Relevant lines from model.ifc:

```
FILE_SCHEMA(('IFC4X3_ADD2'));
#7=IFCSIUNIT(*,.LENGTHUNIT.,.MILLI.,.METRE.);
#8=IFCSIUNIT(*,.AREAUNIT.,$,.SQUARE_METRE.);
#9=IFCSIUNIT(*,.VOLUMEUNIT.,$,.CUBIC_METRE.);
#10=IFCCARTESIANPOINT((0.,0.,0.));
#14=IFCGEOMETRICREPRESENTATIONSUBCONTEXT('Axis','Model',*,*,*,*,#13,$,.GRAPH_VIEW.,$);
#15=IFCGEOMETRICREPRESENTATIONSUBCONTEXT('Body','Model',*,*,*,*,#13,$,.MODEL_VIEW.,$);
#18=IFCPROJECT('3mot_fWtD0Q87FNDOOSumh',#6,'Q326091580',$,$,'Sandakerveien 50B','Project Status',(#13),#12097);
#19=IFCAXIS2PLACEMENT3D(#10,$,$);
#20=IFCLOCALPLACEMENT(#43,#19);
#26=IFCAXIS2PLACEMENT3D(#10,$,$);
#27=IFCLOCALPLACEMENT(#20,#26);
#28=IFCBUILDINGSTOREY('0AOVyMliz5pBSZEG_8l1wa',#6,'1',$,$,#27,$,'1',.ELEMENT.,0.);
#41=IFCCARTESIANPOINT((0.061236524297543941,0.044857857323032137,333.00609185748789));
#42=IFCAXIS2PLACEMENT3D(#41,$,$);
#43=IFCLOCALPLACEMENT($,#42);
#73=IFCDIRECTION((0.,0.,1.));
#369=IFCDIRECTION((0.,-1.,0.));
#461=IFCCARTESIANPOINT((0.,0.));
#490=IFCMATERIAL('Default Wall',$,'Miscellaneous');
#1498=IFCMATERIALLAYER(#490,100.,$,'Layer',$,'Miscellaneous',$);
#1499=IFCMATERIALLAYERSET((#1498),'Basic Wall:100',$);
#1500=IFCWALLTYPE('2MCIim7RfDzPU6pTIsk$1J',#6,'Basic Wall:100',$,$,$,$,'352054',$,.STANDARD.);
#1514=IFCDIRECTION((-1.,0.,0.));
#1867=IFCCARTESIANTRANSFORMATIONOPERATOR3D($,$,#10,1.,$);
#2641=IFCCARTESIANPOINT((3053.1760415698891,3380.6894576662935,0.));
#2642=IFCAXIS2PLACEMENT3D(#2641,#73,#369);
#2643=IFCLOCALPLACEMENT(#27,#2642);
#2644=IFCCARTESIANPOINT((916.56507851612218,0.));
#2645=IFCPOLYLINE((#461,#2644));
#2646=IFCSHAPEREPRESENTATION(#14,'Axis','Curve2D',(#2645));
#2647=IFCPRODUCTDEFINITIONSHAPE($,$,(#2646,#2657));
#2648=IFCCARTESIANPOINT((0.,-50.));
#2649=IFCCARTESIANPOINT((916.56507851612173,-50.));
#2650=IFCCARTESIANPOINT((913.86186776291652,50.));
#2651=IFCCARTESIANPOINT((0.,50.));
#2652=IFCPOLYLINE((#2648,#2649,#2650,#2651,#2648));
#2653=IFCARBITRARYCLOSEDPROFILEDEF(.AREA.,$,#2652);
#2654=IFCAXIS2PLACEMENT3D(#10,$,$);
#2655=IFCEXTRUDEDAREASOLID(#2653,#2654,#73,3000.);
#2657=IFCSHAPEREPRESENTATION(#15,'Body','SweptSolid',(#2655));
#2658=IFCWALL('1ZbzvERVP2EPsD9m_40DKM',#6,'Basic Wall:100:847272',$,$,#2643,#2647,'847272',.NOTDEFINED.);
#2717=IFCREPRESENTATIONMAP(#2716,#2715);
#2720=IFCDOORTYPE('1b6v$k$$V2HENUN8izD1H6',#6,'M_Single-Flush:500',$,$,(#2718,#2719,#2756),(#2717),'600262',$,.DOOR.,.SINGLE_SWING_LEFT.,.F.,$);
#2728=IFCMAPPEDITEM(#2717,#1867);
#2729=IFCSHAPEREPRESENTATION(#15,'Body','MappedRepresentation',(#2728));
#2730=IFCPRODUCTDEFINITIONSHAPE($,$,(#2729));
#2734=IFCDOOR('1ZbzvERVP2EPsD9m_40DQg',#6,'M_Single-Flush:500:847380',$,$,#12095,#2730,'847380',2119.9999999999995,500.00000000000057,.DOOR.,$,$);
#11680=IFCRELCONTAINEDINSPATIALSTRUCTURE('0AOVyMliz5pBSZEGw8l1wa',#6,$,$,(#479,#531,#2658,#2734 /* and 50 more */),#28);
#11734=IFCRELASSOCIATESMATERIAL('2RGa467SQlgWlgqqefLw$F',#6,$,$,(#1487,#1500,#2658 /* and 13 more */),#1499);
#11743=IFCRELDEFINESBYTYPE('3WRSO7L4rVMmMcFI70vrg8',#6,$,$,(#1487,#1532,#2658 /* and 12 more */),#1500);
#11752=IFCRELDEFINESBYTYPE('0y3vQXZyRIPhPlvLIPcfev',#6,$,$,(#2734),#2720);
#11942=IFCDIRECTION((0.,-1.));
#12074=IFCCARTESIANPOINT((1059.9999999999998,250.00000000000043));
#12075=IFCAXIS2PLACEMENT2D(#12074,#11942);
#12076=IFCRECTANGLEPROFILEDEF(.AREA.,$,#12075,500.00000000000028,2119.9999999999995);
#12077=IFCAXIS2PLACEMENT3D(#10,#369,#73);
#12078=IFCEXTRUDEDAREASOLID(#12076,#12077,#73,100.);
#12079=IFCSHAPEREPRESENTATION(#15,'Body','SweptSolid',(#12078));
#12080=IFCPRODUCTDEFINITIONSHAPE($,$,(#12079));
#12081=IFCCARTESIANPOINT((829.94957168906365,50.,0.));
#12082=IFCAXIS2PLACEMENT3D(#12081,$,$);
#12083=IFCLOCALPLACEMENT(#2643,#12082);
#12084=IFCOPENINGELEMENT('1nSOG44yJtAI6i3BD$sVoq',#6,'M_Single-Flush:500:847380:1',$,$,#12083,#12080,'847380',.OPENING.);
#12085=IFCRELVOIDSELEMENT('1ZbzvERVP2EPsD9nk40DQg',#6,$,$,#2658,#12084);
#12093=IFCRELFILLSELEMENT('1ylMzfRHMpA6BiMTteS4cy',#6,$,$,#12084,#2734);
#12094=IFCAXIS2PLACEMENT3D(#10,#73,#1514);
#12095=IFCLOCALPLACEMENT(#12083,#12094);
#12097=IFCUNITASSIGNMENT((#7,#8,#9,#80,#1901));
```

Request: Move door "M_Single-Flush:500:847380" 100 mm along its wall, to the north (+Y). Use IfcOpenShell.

```python
import ifcopenshell
import ifcopenshell.api.geometry
import ifcopenshell.util.placement
import ifcopenshell.util.unit

model = ifcopenshell.open("model.ifc")
unit_scale = ifcopenshell.util.unit.calculate_unit_scale(model)

door = model.by_guid("1ZbzvERVP2EPsD9m_40DQg")
opening = door.FillsVoids[0].RelatingOpeningElement
wall = opening.VoidsElements[0].RelatingBuildingElement

wall_matrix = ifcopenshell.util.placement.get_local_placement(wall.ObjectPlacement)
shift = wall_matrix[:3, 0] * -0.1 / unit_scale
before = ifcopenshell.util.placement.get_local_placement(door.ObjectPlacement)[:3, 3].copy()

# The door is placed relative to its opening, so it follows when the opening moves.
matrix = ifcopenshell.util.placement.get_local_placement(opening.ObjectPlacement)
matrix[:3, 3] += shift
ifcopenshell.api.geometry.edit_object_placement(
    model, product=opening, matrix=matrix, is_si=False, should_transform_children=True
)

after = ifcopenshell.util.placement.get_local_placement(door.ObjectPlacement)[:3, 3]
print("door moved by", (after - before).round(3) + 0.0)

model.write("model_edited.ifc")
```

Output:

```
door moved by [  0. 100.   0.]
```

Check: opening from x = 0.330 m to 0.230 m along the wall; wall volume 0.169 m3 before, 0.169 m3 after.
